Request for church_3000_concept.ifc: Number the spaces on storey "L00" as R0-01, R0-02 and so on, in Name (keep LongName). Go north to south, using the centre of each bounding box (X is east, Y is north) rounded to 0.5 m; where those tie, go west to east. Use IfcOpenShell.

First a look at what the model holds.

```python
import ifcopenshell
import ifcopenshell.util.element
import ifcopenshell.util.placement

model = ifcopenshell.open("church_3000_concept.ifc")
print(model.schema)
storey = next(s for s in model.by_type("IfcBuildingStorey") if s.Name == "L00")
spaces = [e for e in ifcopenshell.util.element.get_decomposition(storey) if e.is_a("IfcSpace")]
for e in sorted(spaces, key=lambda e: e.id()):
    origin = ifcopenshell.util.placement.get_local_placement(e.ObjectPlacement)[:3, 3]
    print(e.id(), e.Name, e.LongName, origin.round(2) + 0.0, sep=" | ")
```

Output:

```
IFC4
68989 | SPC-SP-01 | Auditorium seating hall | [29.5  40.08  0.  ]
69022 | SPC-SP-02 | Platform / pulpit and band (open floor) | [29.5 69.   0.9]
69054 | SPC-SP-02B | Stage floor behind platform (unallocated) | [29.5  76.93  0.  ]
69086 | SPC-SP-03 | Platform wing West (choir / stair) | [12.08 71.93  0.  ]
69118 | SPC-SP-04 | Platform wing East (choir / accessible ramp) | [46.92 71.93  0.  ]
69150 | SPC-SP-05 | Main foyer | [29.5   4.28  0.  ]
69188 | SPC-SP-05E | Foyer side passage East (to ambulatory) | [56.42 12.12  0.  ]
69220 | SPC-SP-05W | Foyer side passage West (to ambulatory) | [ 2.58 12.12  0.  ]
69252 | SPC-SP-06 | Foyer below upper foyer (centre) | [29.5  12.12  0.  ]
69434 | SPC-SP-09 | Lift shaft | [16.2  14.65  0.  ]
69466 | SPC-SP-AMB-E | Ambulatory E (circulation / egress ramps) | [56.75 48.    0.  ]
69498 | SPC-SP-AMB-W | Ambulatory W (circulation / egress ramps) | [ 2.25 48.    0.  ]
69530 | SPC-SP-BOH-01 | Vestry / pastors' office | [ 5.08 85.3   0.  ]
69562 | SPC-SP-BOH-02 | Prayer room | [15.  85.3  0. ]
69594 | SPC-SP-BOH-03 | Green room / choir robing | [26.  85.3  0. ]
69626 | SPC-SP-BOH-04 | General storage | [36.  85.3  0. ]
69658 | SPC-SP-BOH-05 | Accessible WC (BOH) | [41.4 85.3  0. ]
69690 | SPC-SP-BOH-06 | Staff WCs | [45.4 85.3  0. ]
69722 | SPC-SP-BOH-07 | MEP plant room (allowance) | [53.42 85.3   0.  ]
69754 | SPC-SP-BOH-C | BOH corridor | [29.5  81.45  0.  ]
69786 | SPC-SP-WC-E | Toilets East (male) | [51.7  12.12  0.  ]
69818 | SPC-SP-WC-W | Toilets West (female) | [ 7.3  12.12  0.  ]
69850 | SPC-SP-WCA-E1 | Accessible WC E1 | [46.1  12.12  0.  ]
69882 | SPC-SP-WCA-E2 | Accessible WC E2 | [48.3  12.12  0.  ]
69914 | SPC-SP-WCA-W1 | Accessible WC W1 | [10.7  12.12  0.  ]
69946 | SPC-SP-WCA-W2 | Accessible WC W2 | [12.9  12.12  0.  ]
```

```python
import ifcopenshell
import ifcopenshell.geom
import ifcopenshell.util.element
import ifcopenshell.util.shape

model = ifcopenshell.open("church_3000_concept.ifc")
settings = ifcopenshell.geom.settings()
settings.set("use-world-coords", True)


def centre(element):
    shape = ifcopenshell.geom.create_shape(settings, element)
    return ifcopenshell.util.shape.get_bbox_centroid(shape.geometry)


storey = next(s for s in model.by_type("IfcBuildingStorey") if s.Name == "L00")
spaces = [e for e in ifcopenshell.util.element.get_decomposition(storey) if e.is_a("IfcSpace")]

# Insertion points can sit at a corner or the storey origin, so sort by the geometry (in metres).
centres = {e: centre(e) for e in spaces}
spaces.sort(key=lambda e: (-round(centres[e][1] / 0.5), centres[e][0]))

for i, e in enumerate(spaces, start=1):
    number = f"R0-{i:02d}"
    e.Name = number
    print(e.id(), number)

model.write("church_3000_concept_rev.ifc")
```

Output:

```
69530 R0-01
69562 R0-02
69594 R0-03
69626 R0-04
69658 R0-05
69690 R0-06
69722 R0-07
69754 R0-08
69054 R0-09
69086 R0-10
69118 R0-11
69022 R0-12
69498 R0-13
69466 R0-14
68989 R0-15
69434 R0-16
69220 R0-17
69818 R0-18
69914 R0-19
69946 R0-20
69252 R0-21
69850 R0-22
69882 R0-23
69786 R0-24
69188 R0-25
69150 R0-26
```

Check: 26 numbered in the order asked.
